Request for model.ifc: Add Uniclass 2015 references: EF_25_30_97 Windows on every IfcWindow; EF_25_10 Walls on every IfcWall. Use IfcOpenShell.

First a look at what the model holds.

```python
import ifcopenshell

model = ifcopenshell.open("model.ifc")
print(model.schema)
print("classifications:", [c.Name for c in model.by_type("IfcClassification")])
for ifc_class in ("IfcDoor", "IfcRoof", "IfcStair", "IfcWall", "IfcWindow"):
    print(ifc_class, len(model.by_type(ifc_class)))
```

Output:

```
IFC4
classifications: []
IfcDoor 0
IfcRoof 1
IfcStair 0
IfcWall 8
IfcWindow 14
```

```python
import ifcopenshell
import ifcopenshell.api.classification

model = ifcopenshell.open("model.ifc")

system = ifcopenshell.api.classification.add_classification(model, classification="Uniclass 2015")

codes = {
    "IfcWindow": ("EF_25_30_97", "Windows"),
    "IfcWall": ("EF_25_10", "Walls"),
}
for ifc_class, (code, name) in codes.items():
    products = model.by_type(ifc_class)
    ifcopenshell.api.classification.add_reference(
        model, products=products, classification=system, identification=code, name=name
    )
    print(code, len(products))

model.write("model_rev.ifc")
```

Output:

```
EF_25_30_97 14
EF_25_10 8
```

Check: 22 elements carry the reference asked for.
